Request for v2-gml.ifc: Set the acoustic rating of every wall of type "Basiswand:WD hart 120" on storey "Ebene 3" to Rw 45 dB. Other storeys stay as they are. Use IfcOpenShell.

First a look at what the model holds.

```python
import ifcopenshell
import ifcopenshell.util.element

model = ifcopenshell.open("v2-gml.ifc")
print(model.schema)
storey = next(s for s in model.by_type("IfcBuildingStorey") if s.Name == "Ebene 3")
walls = [e for e in ifcopenshell.util.element.get_decomposition(storey) if e.is_a("IfcWall")]
seen = {}
for e in walls:
    element_type = ifcopenshell.util.element.get_type(e)
    key = (element_type.Name if element_type != e and element_type else None, ifcopenshell.util.element.get_pset(e, "Pset_WallCommon", "AcousticRating"))
    seen[key] = seen.get(key, 0) + 1
for (name, value), count in sorted(seen.items(), key=str):
    print(count, "x", name, "|", value)
```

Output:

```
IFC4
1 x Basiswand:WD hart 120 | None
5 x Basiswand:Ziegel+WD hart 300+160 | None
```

```python
import ifcopenshell
import ifcopenshell.api.pset
import ifcopenshell.util.element

model = ifcopenshell.open("v2-gml.ifc")

storey = next(s for s in model.by_type("IfcBuildingStorey") if s.Name == "Ebene 3")
walls = [e for e in ifcopenshell.util.element.get_decomposition(storey) if e.is_a("IfcWall")]

count = 0
for e in walls:
    element_type = ifcopenshell.util.element.get_type(e)
    if element_type in (None, e) or element_type.Name != "Basiswand:WD hart 120":
        continue
    # add_pset returns the element's existing set when there is one.
    pset = ifcopenshell.api.pset.add_pset(model, product=e, name="Pset_WallCommon")
    ifcopenshell.api.pset.edit_pset(model, pset=pset, properties={"AcousticRating": "Rw 45 dB"})
    count += 1

print(count, "walls updated")

model.write("v2-gml-out.ifc")
```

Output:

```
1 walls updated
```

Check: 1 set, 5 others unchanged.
